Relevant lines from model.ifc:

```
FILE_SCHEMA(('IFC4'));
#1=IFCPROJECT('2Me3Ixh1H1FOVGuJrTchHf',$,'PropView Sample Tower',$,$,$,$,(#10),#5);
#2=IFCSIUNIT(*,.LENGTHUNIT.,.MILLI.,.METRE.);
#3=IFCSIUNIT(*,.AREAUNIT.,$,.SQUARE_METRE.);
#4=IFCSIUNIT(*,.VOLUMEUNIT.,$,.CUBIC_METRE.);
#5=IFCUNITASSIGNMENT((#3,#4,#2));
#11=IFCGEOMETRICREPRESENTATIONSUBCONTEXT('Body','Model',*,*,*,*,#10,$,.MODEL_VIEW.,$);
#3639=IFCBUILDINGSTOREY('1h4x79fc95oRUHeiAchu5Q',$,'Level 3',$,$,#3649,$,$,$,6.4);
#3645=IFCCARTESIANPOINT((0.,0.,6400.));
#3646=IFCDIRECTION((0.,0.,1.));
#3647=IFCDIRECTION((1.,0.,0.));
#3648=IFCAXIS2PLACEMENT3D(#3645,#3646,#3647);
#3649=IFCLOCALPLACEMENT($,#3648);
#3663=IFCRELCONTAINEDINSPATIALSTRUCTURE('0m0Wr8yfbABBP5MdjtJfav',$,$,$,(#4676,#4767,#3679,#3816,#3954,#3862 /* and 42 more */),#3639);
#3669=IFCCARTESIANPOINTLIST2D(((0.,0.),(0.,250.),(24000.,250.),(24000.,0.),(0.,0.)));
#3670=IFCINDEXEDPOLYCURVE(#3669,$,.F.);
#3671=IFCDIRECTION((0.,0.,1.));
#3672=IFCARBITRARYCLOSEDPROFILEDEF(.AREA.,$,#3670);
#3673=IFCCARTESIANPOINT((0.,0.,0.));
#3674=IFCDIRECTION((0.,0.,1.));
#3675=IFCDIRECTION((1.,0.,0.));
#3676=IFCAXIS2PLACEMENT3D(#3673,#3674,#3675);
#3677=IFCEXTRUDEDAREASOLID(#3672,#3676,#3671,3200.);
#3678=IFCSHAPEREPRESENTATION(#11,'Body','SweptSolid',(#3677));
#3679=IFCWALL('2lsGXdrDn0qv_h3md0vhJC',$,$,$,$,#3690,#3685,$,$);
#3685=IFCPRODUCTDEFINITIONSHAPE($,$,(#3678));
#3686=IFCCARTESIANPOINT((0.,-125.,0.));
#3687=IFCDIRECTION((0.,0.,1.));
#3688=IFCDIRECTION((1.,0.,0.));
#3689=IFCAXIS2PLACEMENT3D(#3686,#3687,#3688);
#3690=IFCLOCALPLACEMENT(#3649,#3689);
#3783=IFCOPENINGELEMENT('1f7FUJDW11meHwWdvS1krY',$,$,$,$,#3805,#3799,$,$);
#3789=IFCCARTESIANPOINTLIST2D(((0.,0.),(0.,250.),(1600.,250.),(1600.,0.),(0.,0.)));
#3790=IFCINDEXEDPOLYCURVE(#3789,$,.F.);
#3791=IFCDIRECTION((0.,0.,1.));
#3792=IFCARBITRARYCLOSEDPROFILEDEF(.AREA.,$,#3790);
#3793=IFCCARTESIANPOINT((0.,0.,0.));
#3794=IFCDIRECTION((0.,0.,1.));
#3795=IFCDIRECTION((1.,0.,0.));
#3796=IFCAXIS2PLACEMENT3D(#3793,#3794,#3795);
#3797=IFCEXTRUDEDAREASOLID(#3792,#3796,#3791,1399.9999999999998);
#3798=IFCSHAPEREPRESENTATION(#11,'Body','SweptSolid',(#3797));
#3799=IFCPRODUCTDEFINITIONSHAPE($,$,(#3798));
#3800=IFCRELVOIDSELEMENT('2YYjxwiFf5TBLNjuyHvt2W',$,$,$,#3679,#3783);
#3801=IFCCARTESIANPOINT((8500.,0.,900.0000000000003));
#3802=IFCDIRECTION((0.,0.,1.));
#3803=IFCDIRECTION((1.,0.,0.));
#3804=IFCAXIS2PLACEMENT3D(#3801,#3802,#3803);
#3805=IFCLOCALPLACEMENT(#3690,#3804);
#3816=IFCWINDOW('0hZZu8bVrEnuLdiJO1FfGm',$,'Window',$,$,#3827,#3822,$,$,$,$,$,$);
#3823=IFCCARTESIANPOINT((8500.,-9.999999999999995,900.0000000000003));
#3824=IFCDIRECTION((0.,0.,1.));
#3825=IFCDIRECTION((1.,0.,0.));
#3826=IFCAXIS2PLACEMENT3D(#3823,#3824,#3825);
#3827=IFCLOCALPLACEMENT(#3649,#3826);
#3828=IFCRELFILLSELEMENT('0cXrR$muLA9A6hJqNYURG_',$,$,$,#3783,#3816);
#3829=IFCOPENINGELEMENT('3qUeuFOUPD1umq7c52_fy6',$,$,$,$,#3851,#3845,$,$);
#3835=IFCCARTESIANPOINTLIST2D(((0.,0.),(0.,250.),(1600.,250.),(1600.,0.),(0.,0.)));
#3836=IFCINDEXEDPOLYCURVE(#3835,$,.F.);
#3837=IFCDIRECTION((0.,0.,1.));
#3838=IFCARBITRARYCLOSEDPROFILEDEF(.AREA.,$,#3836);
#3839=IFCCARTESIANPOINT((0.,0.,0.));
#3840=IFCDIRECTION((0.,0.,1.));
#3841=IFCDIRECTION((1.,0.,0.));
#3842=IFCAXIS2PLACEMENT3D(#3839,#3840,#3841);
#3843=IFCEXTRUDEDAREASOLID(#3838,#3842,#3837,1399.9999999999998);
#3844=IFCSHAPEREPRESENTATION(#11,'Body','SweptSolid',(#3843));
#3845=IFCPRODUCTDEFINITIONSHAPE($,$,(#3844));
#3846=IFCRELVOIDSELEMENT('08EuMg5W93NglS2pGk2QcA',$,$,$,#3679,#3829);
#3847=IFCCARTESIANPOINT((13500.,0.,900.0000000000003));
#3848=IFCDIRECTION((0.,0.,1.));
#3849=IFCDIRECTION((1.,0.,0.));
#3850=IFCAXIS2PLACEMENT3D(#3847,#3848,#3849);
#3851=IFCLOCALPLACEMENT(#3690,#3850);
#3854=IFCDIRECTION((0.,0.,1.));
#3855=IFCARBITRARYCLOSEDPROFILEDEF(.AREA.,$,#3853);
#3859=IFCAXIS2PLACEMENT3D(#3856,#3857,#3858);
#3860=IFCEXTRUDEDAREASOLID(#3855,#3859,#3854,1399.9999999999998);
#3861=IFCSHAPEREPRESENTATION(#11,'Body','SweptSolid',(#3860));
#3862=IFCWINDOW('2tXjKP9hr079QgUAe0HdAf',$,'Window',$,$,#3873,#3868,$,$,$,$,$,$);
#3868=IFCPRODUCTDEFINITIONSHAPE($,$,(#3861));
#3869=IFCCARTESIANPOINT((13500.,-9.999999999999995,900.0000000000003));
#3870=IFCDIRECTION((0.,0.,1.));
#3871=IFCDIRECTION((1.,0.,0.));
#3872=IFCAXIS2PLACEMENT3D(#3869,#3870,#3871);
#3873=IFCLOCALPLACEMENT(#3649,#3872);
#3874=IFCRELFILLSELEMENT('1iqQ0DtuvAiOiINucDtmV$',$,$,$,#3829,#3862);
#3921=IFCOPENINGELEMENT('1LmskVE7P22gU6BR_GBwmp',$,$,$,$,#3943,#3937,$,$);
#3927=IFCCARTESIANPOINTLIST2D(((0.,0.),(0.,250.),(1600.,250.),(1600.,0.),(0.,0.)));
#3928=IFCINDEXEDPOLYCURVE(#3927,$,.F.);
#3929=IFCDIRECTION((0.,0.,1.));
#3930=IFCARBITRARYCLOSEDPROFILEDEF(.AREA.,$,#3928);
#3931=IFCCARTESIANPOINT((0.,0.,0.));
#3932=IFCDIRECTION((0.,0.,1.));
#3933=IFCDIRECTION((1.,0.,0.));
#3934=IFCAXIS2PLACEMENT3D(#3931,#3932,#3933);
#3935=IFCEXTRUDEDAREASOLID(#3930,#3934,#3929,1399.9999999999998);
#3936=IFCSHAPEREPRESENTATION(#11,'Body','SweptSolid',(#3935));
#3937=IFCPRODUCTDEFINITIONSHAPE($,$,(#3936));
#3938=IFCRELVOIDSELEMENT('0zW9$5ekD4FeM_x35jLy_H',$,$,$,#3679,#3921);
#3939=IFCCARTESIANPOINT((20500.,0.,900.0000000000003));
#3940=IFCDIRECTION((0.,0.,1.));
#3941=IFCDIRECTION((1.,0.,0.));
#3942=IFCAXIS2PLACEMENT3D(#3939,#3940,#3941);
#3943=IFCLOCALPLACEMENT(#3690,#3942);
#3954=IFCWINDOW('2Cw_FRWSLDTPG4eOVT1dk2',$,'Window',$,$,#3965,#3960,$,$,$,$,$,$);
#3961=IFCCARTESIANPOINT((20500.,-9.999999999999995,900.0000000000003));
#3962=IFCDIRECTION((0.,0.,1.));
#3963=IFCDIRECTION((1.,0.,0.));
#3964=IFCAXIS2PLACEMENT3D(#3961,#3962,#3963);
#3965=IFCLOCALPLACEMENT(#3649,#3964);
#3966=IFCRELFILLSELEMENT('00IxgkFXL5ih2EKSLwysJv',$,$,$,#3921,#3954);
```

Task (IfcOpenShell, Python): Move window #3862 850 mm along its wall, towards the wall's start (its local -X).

```python
import ifcopenshell
import ifcopenshell.api.geometry
import ifcopenshell.util.placement
import ifcopenshell.util.unit

model = ifcopenshell.open("model.ifc")
unit_scale = ifcopenshell.util.unit.calculate_unit_scale(model)

window = model.by_id(3862)
opening = window.FillsVoids[0].RelatingOpeningElement
wall = opening.VoidsElements[0].RelatingBuildingElement

wall_matrix = ifcopenshell.util.placement.get_local_placement(wall.ObjectPlacement)
shift = wall_matrix[:3, 0] * -0.85 / unit_scale
before = ifcopenshell.util.placement.get_local_placement(window.ObjectPlacement)[:3, 3].copy()

# The window is not placed relative to its opening, so move both.
for product in (opening, window):
    matrix = ifcopenshell.util.placement.get_local_placement(product.ObjectPlacement)
    matrix[:3, 3] += shift
    ifcopenshell.api.geometry.edit_object_placement(model, product=product, matrix=matrix, is_si=False)

after = ifcopenshell.util.placement.get_local_placement(window.ObjectPlacement)[:3, 3]
print("window moved by", (after - before).round(3) + 0.0)

model.write("model_v2.ifc")
```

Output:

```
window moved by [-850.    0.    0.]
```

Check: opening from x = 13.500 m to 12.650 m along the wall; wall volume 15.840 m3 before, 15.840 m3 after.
